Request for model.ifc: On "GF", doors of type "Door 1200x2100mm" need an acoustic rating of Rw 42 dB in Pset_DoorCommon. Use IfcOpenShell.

First a look at what the model holds.

```python
import ifcopenshell
import ifcopenshell.util.element

model = ifcopenshell.open("model.ifc")
print(model.schema)
storey = next(s for s in model.by_type("IfcBuildingStorey") if s.Name == "GF")
doors = [e for e in ifcopenshell.util.element.get_decomposition(storey) if e.is_a("IfcDoor")]
seen = {}
for e in doors:
    element_type = ifcopenshell.util.element.get_type(e)
    key = (element_type.Name if element_type != e and element_type else None, ifcopenshell.util.element.get_pset(e, "Pset_DoorCommon", "AcousticRating"))
    seen[key] = seen.get(key, 0) + 1
for (name, value), count in sorted(seen.items(), key=str):
    print(count, "x", name, "|", value)
```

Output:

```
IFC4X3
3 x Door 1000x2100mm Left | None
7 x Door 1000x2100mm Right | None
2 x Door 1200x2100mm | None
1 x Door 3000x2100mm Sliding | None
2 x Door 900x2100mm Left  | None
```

```python
import ifcopenshell
import ifcopenshell.api.pset
import ifcopenshell.util.element

model = ifcopenshell.open("model.ifc")

storey = next(s for s in model.by_type("IfcBuildingStorey") if s.Name == "GF")
doors = [e for e in ifcopenshell.util.element.get_decomposition(storey) if e.is_a("IfcDoor")]

count = 0
for e in doors:
    element_type = ifcopenshell.util.element.get_type(e)
    if element_type in (None, e) or element_type.Name != "Door 1200x2100mm":
        continue
    # add_pset returns the element's existing set when there is one.
    pset = ifcopenshell.api.pset.add_pset(model, product=e, name="Pset_DoorCommon")
    ifcopenshell.api.pset.edit_pset(model, pset=pset, properties={"AcousticRating": "Rw 42 dB"})
    count += 1

print(count, "doors updated")

model.write("model-out.ifc")
```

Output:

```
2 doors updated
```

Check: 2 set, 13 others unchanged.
